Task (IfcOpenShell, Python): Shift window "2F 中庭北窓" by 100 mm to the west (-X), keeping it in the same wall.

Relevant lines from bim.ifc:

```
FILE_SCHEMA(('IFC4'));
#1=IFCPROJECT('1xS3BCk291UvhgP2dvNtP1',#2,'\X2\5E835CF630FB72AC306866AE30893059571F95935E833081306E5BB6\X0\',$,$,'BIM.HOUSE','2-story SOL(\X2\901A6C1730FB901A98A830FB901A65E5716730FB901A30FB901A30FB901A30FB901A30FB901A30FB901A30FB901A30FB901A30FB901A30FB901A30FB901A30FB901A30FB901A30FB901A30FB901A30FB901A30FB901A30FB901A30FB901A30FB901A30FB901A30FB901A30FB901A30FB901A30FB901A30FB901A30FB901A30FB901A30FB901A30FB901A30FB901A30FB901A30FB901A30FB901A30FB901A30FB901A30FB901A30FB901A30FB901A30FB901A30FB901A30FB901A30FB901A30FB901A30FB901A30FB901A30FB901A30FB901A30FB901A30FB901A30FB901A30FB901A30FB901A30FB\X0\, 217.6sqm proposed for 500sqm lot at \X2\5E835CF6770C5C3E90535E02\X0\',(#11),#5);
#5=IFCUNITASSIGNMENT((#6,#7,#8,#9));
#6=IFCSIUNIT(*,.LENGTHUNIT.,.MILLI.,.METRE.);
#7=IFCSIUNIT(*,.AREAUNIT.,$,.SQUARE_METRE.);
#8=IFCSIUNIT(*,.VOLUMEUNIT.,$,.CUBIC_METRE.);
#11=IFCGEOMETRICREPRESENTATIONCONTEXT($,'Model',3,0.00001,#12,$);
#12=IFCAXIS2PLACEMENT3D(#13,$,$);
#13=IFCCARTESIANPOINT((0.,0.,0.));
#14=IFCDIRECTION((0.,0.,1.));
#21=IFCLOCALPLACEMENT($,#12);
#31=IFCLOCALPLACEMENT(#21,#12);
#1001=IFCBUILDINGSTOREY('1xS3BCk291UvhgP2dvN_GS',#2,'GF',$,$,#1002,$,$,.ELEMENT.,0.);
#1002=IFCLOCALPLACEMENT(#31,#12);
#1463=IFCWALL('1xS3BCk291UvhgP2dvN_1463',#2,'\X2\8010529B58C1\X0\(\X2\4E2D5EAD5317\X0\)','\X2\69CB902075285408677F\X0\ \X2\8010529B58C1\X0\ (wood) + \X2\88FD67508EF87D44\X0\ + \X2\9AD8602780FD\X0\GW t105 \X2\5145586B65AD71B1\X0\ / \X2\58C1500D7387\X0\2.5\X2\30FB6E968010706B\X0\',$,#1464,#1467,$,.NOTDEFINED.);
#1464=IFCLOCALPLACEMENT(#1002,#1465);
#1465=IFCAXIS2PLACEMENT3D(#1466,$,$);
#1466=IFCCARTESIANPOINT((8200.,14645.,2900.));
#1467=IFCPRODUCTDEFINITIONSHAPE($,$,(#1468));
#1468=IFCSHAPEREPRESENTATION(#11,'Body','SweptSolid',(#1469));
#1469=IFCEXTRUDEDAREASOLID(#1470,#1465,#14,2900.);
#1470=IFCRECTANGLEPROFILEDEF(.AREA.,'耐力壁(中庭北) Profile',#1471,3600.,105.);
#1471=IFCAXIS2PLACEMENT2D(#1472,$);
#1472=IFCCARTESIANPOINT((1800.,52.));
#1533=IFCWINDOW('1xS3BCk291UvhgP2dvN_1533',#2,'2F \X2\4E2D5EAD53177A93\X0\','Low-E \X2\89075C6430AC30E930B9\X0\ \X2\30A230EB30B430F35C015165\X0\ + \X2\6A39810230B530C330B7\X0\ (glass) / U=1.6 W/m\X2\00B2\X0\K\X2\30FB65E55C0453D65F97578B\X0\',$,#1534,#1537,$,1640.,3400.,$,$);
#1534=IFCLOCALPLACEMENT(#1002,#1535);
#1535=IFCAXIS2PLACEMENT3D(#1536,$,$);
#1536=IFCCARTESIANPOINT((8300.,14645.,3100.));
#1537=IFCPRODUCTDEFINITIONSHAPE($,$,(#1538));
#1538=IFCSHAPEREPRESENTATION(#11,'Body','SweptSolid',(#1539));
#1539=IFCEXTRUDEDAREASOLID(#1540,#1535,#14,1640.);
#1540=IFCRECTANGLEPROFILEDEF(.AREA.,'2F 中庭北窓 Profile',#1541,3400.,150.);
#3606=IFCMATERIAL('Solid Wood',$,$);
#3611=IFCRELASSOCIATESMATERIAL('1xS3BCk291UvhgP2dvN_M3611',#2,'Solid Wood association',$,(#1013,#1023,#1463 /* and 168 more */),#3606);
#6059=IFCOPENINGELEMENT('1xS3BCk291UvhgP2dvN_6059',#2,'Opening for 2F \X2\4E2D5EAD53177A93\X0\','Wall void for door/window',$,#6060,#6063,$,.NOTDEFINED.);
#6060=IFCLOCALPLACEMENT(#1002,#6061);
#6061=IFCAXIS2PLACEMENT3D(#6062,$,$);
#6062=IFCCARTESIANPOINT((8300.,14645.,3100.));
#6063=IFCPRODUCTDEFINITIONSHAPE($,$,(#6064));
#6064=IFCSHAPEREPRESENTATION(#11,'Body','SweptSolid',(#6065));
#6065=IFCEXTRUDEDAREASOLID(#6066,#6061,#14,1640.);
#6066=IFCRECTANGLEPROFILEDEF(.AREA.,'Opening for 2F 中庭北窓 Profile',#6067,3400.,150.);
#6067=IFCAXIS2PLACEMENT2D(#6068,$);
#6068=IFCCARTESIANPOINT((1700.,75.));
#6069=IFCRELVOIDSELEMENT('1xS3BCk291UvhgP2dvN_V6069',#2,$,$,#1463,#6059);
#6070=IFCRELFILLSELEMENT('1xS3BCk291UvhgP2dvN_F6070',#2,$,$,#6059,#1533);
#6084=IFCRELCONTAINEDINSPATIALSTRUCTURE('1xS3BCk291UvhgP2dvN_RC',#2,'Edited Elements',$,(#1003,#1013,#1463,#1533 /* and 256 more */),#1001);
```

```python
import ifcopenshell
import ifcopenshell.api.geometry
import ifcopenshell.util.placement
import ifcopenshell.util.unit

model = ifcopenshell.open("bim.ifc")
unit_scale = ifcopenshell.util.unit.calculate_unit_scale(model)

window = model.by_id(1533)
opening = window.FillsVoids[0].RelatingOpeningElement
wall = opening.VoidsElements[0].RelatingBuildingElement

wall_matrix = ifcopenshell.util.placement.get_local_placement(wall.ObjectPlacement)
shift = wall_matrix[:3, 0] * -0.1 / unit_scale
before = ifcopenshell.util.placement.get_local_placement(window.ObjectPlacement)[:3, 3].copy()

# The window is not placed relative to its opening, so move both.
for product in (opening, window):
    matrix = ifcopenshell.util.placement.get_local_placement(product.ObjectPlacement)
    matrix[:3, 3] += shift
    ifcopenshell.api.geometry.edit_object_placement(model, product=product, matrix=matrix, is_si=False)

after = ifcopenshell.util.placement.get_local_placement(window.ObjectPlacement)[:3, 3]
print("window moved by", (after - before).round(3) + 0.0)

model.write("bim_edited.ifc")
```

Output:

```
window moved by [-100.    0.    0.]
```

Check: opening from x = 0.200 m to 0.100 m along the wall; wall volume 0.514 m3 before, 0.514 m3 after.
